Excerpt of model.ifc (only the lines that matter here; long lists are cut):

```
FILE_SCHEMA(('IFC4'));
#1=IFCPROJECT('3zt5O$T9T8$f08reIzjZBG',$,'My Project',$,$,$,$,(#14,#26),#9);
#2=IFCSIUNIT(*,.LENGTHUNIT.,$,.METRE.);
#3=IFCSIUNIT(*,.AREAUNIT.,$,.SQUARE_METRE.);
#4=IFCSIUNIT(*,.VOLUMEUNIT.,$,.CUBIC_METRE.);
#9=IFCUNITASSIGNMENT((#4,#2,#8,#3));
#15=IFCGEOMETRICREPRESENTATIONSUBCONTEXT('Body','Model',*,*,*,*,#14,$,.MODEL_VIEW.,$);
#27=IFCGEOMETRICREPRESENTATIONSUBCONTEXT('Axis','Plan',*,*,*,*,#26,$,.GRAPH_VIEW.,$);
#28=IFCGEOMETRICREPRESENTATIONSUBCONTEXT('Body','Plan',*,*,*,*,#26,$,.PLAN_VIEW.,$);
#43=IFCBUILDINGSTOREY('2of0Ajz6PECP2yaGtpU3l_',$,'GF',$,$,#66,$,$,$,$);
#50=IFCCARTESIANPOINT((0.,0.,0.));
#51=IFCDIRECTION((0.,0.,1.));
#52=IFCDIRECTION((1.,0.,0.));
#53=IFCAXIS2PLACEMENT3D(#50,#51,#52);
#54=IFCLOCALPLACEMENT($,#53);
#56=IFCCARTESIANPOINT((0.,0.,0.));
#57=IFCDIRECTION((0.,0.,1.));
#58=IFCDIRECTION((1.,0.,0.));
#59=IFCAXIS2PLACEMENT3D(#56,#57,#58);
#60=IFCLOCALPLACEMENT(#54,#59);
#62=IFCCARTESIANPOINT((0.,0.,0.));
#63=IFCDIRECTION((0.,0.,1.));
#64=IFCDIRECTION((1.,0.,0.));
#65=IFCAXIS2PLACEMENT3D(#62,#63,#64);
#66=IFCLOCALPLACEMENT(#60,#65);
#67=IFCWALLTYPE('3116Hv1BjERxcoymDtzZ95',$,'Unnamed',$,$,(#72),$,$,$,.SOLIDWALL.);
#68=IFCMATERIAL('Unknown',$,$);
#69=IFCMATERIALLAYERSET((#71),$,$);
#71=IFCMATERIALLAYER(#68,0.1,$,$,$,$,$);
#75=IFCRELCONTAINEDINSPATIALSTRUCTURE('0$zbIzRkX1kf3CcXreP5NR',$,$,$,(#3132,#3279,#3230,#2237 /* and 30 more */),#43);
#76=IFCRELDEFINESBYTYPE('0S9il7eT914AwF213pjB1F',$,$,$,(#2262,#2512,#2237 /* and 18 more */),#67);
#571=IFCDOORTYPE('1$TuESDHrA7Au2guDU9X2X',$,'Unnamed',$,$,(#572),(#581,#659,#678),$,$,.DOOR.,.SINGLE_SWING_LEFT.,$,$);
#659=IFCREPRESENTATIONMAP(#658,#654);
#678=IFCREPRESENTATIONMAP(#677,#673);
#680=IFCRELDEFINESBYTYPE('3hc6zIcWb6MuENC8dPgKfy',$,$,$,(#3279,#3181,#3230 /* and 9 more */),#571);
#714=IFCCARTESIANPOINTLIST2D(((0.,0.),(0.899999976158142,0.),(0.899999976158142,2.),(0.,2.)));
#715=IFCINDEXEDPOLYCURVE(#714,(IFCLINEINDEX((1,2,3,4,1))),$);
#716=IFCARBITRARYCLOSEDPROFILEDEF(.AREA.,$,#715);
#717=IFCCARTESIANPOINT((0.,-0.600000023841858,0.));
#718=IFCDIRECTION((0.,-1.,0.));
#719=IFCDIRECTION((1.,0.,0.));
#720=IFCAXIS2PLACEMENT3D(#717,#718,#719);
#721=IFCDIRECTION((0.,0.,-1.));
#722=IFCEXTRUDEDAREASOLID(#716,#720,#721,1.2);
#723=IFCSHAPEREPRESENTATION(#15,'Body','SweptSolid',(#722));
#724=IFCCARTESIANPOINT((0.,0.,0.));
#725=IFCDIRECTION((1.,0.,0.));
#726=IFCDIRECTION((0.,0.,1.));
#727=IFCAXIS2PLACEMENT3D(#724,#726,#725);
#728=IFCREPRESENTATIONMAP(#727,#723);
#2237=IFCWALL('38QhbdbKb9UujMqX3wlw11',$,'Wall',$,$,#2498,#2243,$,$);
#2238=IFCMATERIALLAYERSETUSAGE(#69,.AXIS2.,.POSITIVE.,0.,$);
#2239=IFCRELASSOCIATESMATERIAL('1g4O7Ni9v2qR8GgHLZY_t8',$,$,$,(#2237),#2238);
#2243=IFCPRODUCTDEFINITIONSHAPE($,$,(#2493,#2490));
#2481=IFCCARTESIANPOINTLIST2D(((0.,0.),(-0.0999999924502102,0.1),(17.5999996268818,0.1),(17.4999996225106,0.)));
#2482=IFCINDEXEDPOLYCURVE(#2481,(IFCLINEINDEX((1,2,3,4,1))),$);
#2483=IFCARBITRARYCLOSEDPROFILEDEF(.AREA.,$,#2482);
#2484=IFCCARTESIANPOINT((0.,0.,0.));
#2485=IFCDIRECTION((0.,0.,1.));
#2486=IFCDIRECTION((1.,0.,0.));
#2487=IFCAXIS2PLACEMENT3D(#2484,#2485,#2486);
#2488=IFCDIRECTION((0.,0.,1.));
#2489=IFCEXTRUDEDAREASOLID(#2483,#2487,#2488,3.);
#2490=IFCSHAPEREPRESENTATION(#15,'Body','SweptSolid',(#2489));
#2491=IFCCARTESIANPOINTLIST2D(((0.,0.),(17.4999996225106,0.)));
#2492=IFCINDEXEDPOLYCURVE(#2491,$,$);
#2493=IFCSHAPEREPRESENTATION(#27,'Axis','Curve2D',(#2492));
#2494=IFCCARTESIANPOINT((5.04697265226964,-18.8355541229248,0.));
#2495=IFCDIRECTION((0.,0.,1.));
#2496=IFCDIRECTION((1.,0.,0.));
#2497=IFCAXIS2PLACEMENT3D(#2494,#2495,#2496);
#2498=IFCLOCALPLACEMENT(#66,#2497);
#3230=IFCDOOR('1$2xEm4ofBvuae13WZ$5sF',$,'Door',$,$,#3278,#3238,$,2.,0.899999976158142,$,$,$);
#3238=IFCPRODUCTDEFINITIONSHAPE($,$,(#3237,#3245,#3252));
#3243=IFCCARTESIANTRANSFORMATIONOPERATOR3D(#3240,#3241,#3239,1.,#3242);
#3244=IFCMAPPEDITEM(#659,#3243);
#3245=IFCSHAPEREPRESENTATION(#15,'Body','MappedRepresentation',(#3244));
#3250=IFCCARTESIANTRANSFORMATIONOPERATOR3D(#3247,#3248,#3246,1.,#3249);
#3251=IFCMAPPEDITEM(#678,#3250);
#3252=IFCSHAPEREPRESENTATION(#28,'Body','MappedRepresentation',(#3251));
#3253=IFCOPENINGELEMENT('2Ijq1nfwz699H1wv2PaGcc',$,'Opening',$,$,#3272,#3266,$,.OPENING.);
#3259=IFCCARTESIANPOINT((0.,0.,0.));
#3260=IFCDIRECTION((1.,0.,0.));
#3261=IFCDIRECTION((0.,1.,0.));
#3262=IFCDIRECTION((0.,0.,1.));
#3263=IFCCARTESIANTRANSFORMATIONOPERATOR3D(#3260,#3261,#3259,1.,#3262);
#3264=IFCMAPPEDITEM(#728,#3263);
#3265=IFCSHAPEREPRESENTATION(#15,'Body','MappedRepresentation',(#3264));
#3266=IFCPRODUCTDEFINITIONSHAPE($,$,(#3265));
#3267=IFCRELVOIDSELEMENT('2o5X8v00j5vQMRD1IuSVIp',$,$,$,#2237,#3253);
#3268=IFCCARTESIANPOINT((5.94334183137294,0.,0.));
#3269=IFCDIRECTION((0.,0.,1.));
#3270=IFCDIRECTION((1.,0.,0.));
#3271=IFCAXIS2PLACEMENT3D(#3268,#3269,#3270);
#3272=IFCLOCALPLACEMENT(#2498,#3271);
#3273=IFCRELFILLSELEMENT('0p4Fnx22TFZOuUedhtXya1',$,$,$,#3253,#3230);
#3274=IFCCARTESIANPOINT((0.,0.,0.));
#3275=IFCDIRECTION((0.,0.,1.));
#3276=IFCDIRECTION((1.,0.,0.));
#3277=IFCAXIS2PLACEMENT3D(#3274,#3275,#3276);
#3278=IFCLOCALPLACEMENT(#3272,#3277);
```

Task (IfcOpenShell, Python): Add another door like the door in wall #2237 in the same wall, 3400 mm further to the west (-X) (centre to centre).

```python
import ifcopenshell
import ifcopenshell.api.feature
import ifcopenshell.api.geometry
import ifcopenshell.api.root
import ifcopenshell.geom
import ifcopenshell.util.element
import ifcopenshell.util.placement
import ifcopenshell.util.shape

model = ifcopenshell.open("model.ifc")
settings = ifcopenshell.geom.settings()


def volume(element):
    """Net volume in cubic metres, openings subtracted."""
    shape = ifcopenshell.geom.create_shape(settings, element)
    return ifcopenshell.util.shape.get_volume(shape.geometry)


door = model.by_id(3230)
opening = door.FillsVoids[0].RelatingOpeningElement
wall = opening.VoidsElements[0].RelatingBuildingElement
before = volume(wall)
shift = ifcopenshell.util.placement.get_local_placement(wall.ObjectPlacement)[:3, 0] * -3.4

# copy_class copies the void relationship, type, container and properties, but no geometry.
new_opening = ifcopenshell.api.root.copy_class(model, product=opening)
new_opening.Representation = ifcopenshell.util.element.copy_deep(
    model, opening.Representation, exclude=["IfcGeometricRepresentationContext", "IfcRepresentationMap"]
)
new_door = ifcopenshell.api.root.copy_class(model, product=door)
new_door.Representation = ifcopenshell.util.element.copy_deep(
    model, door.Representation, exclude=["IfcGeometricRepresentationContext", "IfcRepresentationMap"]
)
ifcopenshell.api.feature.add_filling(model, opening=new_opening, element=new_door)

for old, new in ((opening, new_opening), (door, new_door)):
    matrix = ifcopenshell.util.placement.get_local_placement(old.ObjectPlacement)
    matrix[:3, 3] += shift
    ifcopenshell.api.geometry.edit_object_placement(model, product=new, matrix=matrix, is_si=False)

after = volume(wall)

print(f"wall volume {before:.3f} -> {after:.3f} m3")

model.write("model_updated.ifc")
```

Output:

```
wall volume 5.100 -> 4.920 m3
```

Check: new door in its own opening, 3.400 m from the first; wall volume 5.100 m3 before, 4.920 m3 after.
